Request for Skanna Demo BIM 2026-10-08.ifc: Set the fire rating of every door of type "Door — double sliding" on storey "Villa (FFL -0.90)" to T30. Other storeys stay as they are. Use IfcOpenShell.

First a look at what the model holds.

```python
import ifcopenshell
import ifcopenshell.util.element

model = ifcopenshell.open("Skanna Demo BIM 2026-10-08.ifc")
print(model.schema)
storey = next(s for s in model.by_type("IfcBuildingStorey") if s.Name == "Villa (FFL -0.90)")
doors = [e for e in ifcopenshell.util.element.get_decomposition(storey) if e.is_a("IfcDoor")]
seen = {}
for e in doors:
    element_type = ifcopenshell.util.element.get_type(e)
    key = (element_type.Name if element_type != e and element_type else None, ifcopenshell.util.element.get_pset(e, "Pset_DoorCommon", "FireRating"))
    seen[key] = seen.get(key, 0) + 1
for (name, value), count in sorted(seen.items(), key=str):
    print(count, "x", name, "|", value)
```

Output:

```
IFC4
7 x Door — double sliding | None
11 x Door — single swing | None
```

```python
import ifcopenshell
import ifcopenshell.api.pset
import ifcopenshell.util.element

model = ifcopenshell.open("Skanna Demo BIM 2026-10-08.ifc")

storey = next(s for s in model.by_type("IfcBuildingStorey") if s.Name == "Villa (FFL -0.90)")
doors = [e for e in ifcopenshell.util.element.get_decomposition(storey) if e.is_a("IfcDoor")]

count = 0
for e in doors:
    element_type = ifcopenshell.util.element.get_type(e)
    if element_type in (None, e) or element_type.Name != "Door — double sliding":
        continue
    # add_pset returns the element's existing set when there is one.
    pset = ifcopenshell.api.pset.add_pset(model, product=e, name="Pset_DoorCommon")
    ifcopenshell.api.pset.edit_pset(model, pset=pset, properties={"FireRating": "T30"})
    count += 1

print(count, "doors updated")

model.write("Skanna Demo BIM 2026-10-08_updated.ifc")
```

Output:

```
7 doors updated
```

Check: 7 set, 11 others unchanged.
